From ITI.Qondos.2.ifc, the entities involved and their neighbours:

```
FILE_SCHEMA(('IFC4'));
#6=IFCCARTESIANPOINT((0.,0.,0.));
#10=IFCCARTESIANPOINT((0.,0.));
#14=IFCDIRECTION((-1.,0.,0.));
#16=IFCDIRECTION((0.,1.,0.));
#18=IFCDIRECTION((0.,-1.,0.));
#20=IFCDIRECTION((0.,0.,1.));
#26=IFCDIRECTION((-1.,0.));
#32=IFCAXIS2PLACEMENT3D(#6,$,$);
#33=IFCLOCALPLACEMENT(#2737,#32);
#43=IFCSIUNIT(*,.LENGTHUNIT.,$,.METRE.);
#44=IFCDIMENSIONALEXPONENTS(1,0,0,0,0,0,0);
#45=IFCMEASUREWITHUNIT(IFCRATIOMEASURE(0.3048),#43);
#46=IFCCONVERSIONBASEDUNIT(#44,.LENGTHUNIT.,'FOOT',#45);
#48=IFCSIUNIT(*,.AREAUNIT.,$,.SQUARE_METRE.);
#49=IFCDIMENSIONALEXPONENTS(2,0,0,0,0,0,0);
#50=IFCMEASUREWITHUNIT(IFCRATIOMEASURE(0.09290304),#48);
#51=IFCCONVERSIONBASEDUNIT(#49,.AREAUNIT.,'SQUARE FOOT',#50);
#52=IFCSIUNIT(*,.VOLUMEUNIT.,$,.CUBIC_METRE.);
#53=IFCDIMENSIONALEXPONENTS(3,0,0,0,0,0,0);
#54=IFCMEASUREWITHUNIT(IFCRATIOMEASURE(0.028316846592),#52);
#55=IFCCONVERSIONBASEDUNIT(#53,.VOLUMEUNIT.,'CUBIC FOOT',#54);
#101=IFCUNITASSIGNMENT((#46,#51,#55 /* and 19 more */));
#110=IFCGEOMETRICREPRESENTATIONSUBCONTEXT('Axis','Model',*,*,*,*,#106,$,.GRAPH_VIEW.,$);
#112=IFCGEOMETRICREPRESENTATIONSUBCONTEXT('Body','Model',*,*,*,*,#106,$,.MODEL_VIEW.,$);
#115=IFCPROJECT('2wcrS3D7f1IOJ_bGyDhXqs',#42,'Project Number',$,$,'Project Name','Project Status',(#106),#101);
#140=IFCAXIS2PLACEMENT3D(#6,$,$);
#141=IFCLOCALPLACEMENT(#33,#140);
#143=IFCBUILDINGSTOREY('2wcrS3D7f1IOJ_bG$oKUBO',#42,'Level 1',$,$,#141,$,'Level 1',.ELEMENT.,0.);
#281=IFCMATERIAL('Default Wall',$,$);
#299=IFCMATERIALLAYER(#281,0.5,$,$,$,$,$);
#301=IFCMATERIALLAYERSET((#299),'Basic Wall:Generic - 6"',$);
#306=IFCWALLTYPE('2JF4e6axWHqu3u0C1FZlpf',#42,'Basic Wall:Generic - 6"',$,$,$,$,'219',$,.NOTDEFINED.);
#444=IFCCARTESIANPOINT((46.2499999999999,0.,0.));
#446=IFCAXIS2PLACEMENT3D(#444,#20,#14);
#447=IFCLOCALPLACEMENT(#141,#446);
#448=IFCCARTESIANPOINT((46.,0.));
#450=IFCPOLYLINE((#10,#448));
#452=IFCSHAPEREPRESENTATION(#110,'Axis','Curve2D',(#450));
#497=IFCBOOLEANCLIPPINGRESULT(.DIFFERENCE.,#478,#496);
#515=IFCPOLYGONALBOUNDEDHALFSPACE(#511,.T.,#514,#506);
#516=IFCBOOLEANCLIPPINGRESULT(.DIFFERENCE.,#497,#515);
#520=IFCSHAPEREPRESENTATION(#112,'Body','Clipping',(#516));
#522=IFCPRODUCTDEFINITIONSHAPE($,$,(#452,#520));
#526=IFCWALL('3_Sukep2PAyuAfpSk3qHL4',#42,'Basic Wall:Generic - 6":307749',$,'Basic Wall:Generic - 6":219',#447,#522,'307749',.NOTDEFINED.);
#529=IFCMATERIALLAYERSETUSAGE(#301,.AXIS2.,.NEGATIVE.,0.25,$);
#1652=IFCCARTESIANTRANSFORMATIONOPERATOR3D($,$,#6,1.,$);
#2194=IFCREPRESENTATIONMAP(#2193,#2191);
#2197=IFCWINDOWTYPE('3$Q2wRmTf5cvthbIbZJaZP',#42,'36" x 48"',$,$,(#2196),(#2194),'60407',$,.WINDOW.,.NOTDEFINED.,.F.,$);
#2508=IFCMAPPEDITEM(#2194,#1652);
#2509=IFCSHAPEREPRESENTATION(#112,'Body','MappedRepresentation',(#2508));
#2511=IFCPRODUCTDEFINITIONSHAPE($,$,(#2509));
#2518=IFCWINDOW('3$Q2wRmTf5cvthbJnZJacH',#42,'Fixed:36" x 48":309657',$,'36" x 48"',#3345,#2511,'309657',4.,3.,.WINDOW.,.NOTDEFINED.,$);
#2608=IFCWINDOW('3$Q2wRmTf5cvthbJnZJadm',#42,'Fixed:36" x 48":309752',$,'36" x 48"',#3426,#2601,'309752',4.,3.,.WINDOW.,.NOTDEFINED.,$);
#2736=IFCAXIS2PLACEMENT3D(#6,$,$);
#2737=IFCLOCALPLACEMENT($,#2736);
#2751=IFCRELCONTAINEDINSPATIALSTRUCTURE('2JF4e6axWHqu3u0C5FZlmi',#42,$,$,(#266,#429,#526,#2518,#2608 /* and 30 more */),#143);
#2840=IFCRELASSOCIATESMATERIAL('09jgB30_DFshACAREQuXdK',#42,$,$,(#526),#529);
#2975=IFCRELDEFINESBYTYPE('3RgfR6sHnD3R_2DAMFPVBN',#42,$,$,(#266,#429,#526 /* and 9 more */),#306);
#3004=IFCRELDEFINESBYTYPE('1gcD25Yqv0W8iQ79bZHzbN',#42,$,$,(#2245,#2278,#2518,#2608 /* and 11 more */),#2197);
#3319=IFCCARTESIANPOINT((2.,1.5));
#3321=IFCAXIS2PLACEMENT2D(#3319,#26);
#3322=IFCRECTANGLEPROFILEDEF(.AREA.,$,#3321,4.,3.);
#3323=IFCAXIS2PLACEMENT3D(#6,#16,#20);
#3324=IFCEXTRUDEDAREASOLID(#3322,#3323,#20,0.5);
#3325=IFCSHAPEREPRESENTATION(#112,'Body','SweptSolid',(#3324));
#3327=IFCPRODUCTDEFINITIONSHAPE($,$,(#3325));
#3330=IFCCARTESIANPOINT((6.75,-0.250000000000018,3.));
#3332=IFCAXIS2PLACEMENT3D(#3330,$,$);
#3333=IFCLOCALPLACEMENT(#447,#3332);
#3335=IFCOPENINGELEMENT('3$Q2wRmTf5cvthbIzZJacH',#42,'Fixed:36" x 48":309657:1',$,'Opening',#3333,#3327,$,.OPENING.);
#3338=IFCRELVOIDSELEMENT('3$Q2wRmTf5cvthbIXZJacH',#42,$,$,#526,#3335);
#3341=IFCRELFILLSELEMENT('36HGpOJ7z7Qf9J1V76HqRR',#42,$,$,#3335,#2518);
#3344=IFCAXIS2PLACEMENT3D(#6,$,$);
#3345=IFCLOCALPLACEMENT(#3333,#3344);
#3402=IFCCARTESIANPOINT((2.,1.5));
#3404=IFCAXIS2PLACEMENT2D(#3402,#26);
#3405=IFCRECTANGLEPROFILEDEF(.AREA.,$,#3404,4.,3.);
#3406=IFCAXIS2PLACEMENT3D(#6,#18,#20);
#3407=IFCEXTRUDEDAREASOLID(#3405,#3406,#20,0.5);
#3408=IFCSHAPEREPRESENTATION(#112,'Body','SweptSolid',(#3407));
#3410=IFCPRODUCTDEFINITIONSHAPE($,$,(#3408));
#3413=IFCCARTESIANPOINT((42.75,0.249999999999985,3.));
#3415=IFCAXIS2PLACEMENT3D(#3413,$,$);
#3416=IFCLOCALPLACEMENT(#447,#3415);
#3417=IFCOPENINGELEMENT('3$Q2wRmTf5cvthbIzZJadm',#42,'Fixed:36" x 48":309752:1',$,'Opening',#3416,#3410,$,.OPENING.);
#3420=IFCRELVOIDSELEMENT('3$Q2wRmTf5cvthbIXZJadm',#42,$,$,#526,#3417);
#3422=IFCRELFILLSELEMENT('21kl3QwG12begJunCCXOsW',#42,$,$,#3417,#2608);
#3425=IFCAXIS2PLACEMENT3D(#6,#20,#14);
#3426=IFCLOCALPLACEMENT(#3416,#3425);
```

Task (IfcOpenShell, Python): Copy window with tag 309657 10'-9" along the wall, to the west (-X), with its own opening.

```python
import ifcopenshell
import ifcopenshell.api.feature
import ifcopenshell.api.geometry
import ifcopenshell.api.root
import ifcopenshell.geom
import ifcopenshell.util.element
import ifcopenshell.util.placement
import ifcopenshell.util.shape
import ifcopenshell.util.unit

model = ifcopenshell.open("ITI.Qondos.2.ifc")
unit_scale = ifcopenshell.util.unit.calculate_unit_scale(model)
settings = ifcopenshell.geom.settings()


def volume(element):
    """Net volume in cubic metres, openings subtracted."""
    shape = ifcopenshell.geom.create_shape(settings, element)
    return ifcopenshell.util.shape.get_volume(shape.geometry)


def reuse_history(source, copy):
    """copy_class also copies each property set's owner history, people and application; keep the originals."""
    for rel in copy.IsDefinedBy:
        if rel.is_a("IfcRelDefinesByProperties") and (history := rel.RelatingPropertyDefinition.OwnerHistory):
            rel.RelatingPropertyDefinition.OwnerHistory = source.OwnerHistory
            ifcopenshell.util.element.remove_deep2(model, history)


window = model.by_guid("3$Q2wRmTf5cvthbJnZJacH")
opening = window.FillsVoids[0].RelatingOpeningElement
wall = opening.VoidsElements[0].RelatingBuildingElement
before = volume(wall)
shift = ifcopenshell.util.placement.get_local_placement(wall.ObjectPlacement)[:3, 0] * 129 * 0.0254 / unit_scale

# copy_class copies the void relationship, type, container and properties, but no geometry.
new_opening = ifcopenshell.api.root.copy_class(model, product=opening)
new_opening.Representation = ifcopenshell.util.element.copy_deep(
    model, opening.Representation, exclude=["IfcGeometricRepresentationContext", "IfcRepresentationMap"]
)
new_opening.Name = 'Fixed:36" x 48"'
new_window = ifcopenshell.api.root.copy_class(model, product=window)
new_window.Representation = ifcopenshell.util.element.copy_deep(
    model, window.Representation, exclude=["IfcGeometricRepresentationContext", "IfcRepresentationMap"]
)
new_window.Name = 'Fixed:36" x 48"'
new_window.Tag = None
reuse_history(window, new_window)
ifcopenshell.api.feature.add_filling(model, opening=new_opening, element=new_window)

for old, new in ((opening, new_opening), (window, new_window)):
    matrix = ifcopenshell.util.placement.get_local_placement(old.ObjectPlacement)
    matrix[:3, 3] += shift
    ifcopenshell.api.geometry.edit_object_placement(model, product=new, matrix=matrix, is_si=False)

after = volume(wall)

print(f"wall volume {before:.3f} -> {after:.3f} m3")

model.write("ITI.Qondos.2_edited.ifc")
```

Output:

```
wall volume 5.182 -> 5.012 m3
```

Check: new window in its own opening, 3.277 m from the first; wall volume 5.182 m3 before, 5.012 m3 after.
